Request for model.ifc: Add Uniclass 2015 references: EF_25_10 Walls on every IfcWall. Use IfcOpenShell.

First a look at what the model holds.

```python
import ifcopenshell

model = ifcopenshell.open("model.ifc")
print(model.schema)
print("classifications:", [c.Name for c in model.by_type("IfcClassification")])
for ifc_class in ("IfcDoor", "IfcRoof", "IfcStair", "IfcWall", "IfcWindow"):
    print(ifc_class, len(model.by_type(ifc_class)))
```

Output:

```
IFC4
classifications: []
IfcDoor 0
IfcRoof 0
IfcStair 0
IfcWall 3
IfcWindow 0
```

```python
import ifcopenshell
import ifcopenshell.api.classification

model = ifcopenshell.open("model.ifc")

system = ifcopenshell.api.classification.add_classification(model, classification="Uniclass 2015")

codes = {
    "IfcWall": ("EF_25_10", "Walls"),
}
for ifc_class, (code, name) in codes.items():
    products = model.by_type(ifc_class)
    ifcopenshell.api.classification.add_reference(
        model, products=products, classification=system, identification=code, name=name
    )
    print(code, len(products))

model.write("model_updated.ifc")
```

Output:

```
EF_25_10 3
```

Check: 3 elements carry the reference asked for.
